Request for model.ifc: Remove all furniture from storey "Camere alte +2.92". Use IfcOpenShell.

First a look at what the model holds.

```python
import ifcopenshell
import ifcopenshell.util.element

model = ifcopenshell.open("model.ifc")
print(model.schema)
storey = next(s for s in model.by_type("IfcBuildingStorey") if s.Name == "Camere alte +2.92")
furniture = [e for e in ifcopenshell.util.element.get_decomposition(storey) if e.is_a("IfcFurnishingElement")]
seen = {}
for e in furniture:
    element_type = ifcopenshell.util.element.get_type(e)
    name = element_type.Name if element_type not in (None, e) else None
    seen[name] = seen.get(name, 0) + 1
for name, count in sorted(seen.items(), key=str):
    print(count, "x", name)
```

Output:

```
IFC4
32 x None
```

```python
import ifcopenshell
import ifcopenshell.api.root
import ifcopenshell.util.element

model = ifcopenshell.open("model.ifc")

storey = next(s for s in model.by_type("IfcBuildingStorey") if s.Name == "Camere alte +2.92")
furniture = [e for e in ifcopenshell.util.element.get_decomposition(storey) if e.is_a("IfcFurnishingElement")]

for e in furniture:
    ifcopenshell.api.root.remove_product(model, product=e)
print(len(furniture), "removed")

model.write("model_edited.ifc")
```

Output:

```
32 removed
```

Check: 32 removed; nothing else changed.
